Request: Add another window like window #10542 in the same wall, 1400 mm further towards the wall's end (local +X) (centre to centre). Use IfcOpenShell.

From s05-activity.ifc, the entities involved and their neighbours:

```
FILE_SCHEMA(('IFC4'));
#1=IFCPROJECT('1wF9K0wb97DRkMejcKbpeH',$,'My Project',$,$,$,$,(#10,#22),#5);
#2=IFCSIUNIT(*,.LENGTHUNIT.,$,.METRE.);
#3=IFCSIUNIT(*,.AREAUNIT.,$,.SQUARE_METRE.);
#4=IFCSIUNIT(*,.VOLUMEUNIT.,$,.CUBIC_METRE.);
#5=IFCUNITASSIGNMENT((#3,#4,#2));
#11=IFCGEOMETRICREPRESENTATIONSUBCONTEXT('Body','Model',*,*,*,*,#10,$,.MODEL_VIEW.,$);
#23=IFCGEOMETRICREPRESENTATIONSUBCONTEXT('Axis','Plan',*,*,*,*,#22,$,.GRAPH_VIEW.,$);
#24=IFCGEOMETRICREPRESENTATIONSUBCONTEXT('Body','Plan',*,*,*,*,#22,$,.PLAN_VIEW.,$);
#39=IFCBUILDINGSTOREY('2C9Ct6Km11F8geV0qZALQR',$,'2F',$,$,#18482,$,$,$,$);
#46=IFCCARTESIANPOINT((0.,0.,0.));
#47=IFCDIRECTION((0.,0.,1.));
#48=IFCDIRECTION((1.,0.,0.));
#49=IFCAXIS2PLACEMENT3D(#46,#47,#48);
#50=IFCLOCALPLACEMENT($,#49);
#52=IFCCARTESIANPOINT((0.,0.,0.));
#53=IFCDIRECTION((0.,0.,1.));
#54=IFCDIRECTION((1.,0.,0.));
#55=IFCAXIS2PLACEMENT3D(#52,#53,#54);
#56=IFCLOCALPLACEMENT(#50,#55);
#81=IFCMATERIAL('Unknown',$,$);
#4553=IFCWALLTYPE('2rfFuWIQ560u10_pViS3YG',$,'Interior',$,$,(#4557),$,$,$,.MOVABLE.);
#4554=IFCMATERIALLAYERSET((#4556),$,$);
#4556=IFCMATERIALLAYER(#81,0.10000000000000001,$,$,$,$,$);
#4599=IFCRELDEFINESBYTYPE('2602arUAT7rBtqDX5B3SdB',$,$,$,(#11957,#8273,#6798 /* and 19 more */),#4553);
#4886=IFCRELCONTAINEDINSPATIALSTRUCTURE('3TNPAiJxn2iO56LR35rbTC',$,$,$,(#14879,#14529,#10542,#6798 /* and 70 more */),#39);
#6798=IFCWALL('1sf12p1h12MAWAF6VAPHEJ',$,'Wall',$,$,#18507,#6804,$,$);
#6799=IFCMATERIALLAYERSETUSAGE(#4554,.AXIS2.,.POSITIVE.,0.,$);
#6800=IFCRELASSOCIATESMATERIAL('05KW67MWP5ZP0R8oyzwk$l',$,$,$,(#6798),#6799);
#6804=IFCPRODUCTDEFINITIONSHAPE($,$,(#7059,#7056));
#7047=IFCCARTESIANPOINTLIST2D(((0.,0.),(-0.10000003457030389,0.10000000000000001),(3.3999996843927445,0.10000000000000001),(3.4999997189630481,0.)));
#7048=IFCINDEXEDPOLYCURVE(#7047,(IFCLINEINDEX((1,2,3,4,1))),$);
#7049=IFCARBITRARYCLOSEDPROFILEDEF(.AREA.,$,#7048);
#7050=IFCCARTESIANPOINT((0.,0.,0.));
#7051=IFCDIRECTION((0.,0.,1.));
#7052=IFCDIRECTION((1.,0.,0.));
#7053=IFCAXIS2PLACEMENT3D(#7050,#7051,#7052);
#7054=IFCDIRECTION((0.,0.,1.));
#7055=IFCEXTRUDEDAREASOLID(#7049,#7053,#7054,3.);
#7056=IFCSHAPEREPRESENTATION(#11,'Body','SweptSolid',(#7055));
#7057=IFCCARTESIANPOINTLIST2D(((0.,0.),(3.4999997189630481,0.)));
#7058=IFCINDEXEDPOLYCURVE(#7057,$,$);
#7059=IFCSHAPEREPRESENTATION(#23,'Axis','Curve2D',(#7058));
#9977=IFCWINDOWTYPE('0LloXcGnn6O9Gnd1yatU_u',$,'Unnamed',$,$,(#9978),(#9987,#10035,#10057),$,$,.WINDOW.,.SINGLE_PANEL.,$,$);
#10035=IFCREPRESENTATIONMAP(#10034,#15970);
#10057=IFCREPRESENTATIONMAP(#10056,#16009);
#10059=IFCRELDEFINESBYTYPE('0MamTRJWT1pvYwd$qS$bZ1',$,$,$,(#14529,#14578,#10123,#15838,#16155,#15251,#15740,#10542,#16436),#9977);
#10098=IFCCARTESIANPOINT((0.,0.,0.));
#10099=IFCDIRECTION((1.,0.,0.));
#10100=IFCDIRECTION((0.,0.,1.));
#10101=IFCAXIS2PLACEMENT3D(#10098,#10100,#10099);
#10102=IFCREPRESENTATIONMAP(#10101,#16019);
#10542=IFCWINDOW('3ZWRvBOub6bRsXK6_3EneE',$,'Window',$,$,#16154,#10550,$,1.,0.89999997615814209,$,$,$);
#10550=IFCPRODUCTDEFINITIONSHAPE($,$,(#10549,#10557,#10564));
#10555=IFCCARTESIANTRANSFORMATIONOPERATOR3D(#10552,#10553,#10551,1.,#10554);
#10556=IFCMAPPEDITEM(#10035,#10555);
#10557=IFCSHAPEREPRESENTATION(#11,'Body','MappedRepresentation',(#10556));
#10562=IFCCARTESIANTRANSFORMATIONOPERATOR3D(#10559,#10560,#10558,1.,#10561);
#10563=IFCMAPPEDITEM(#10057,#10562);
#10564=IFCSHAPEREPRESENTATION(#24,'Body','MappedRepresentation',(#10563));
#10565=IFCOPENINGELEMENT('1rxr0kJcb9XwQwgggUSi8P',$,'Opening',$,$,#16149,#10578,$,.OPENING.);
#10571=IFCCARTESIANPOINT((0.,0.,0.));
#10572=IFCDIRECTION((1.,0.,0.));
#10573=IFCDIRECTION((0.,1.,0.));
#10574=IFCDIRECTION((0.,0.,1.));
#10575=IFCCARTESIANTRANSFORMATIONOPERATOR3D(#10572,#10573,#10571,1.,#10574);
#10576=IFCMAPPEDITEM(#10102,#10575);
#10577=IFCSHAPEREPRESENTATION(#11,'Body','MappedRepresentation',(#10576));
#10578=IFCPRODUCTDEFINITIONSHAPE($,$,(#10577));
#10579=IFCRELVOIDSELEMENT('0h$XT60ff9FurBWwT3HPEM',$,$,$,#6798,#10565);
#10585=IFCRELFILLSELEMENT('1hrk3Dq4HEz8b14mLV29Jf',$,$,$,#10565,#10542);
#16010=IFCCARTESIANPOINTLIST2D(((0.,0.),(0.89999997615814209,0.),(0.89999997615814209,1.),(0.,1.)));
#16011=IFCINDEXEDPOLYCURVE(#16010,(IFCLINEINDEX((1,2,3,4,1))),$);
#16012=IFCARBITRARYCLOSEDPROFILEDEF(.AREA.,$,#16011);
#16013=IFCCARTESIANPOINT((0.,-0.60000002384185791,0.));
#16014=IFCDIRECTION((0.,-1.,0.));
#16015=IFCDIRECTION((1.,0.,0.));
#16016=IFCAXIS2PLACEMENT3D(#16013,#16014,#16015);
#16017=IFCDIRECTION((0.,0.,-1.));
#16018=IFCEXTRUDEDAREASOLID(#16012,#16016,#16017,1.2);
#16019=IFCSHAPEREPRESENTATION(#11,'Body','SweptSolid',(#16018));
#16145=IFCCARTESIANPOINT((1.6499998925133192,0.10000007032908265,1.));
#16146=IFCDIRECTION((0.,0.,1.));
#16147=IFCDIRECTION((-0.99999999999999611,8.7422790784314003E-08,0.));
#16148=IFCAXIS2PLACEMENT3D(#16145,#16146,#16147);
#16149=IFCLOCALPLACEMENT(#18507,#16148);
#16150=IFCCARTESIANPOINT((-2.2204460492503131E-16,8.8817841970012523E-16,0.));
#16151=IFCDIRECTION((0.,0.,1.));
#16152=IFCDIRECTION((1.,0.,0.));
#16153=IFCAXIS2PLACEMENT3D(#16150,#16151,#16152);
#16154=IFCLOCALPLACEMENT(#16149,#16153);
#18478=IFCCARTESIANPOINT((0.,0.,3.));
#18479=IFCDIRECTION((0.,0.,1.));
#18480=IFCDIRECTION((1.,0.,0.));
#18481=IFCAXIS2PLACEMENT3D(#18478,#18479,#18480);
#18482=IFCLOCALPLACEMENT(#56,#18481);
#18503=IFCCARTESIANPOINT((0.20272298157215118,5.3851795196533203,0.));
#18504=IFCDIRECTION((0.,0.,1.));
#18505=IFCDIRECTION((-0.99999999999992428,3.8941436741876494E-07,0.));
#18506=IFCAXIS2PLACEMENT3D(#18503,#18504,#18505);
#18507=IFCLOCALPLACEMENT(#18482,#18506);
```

```python
import ifcopenshell
import ifcopenshell.api.feature
import ifcopenshell.api.geometry
import ifcopenshell.api.root
import ifcopenshell.geom
import ifcopenshell.util.element
import ifcopenshell.util.placement
import ifcopenshell.util.shape

model = ifcopenshell.open("s05-activity.ifc")
settings = ifcopenshell.geom.settings()


def volume(element):
    """Net volume in cubic metres, openings subtracted."""
    shape = ifcopenshell.geom.create_shape(settings, element)
    return ifcopenshell.util.shape.get_volume(shape.geometry)


window = model.by_guid("3ZWRvBOub6bRsXK6_3EneE")
opening = window.FillsVoids[0].RelatingOpeningElement
wall = opening.VoidsElements[0].RelatingBuildingElement
before = volume(wall)
shift = ifcopenshell.util.placement.get_local_placement(wall.ObjectPlacement)[:3, 0] * 1.4

# copy_class copies the void relationship, type, container and properties, but no geometry.
new_opening = ifcopenshell.api.root.copy_class(model, product=opening)
new_opening.Representation = ifcopenshell.util.element.copy_deep(
    model, opening.Representation, exclude=["IfcGeometricRepresentationContext", "IfcRepresentationMap"]
)
new_window = ifcopenshell.api.root.copy_class(model, product=window)
new_window.Representation = ifcopenshell.util.element.copy_deep(
    model, window.Representation, exclude=["IfcGeometricRepresentationContext", "IfcRepresentationMap"]
)
ifcopenshell.api.feature.add_filling(model, opening=new_opening, element=new_window)

for old, new in ((opening, new_opening), (window, new_window)):
    matrix = ifcopenshell.util.placement.get_local_placement(old.ObjectPlacement)
    matrix[:3, 3] += shift
    ifcopenshell.api.geometry.edit_object_placement(model, product=new, matrix=matrix, is_si=False)

after = volume(wall)

print(f"wall volume {before:.3f} -> {after:.3f} m3")

model.write("s05-activity_v2.ifc")
```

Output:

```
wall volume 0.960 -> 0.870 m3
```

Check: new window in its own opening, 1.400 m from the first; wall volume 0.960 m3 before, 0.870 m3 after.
